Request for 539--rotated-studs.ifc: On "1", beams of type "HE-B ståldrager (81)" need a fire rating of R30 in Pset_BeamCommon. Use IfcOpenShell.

First a look at what the model holds.

```python
import ifcopenshell
import ifcopenshell.util.element

model = ifcopenshell.open("539--rotated-studs.ifc")
print(model.schema)
storey = next(s for s in model.by_type("IfcBuildingStorey") if s.Name == "1")
beams = [e for e in ifcopenshell.util.element.get_decomposition(storey) if e.is_a("IfcBeam")]
seen = {}
for e in beams:
    element_type = ifcopenshell.util.element.get_type(e)
    key = (element_type.Name if element_type != e and element_type else None, ifcopenshell.util.element.get_pset(e, "Pset_BeamCommon", "FireRating"))
    seen[key] = seen.get(key, 0) + 1
for (name, value), count in sorted(seen.items(), key=str):
    print(count, "x", name, "|", value)
```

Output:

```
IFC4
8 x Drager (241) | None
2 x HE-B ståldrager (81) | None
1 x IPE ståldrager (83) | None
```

```python
import ifcopenshell
import ifcopenshell.api.pset
import ifcopenshell.util.element

model = ifcopenshell.open("539--rotated-studs.ifc")

storey = next(s for s in model.by_type("IfcBuildingStorey") if s.Name == "1")
beams = [e for e in ifcopenshell.util.element.get_decomposition(storey) if e.is_a("IfcBeam")]

count = 0
for e in beams:
    element_type = ifcopenshell.util.element.get_type(e)
    if element_type in (None, e) or element_type.Name != "HE-B ståldrager (81)":
        continue
    # add_pset returns the element's existing set when there is one.
    pset = ifcopenshell.api.pset.add_pset(model, product=e, name="Pset_BeamCommon")
    ifcopenshell.api.pset.edit_pset(model, pset=pset, properties={"FireRating": "R30"})
    count += 1

print(count, "beams updated")

model.write("539--rotated-studs_edited.ifc")
```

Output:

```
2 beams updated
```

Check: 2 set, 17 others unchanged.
